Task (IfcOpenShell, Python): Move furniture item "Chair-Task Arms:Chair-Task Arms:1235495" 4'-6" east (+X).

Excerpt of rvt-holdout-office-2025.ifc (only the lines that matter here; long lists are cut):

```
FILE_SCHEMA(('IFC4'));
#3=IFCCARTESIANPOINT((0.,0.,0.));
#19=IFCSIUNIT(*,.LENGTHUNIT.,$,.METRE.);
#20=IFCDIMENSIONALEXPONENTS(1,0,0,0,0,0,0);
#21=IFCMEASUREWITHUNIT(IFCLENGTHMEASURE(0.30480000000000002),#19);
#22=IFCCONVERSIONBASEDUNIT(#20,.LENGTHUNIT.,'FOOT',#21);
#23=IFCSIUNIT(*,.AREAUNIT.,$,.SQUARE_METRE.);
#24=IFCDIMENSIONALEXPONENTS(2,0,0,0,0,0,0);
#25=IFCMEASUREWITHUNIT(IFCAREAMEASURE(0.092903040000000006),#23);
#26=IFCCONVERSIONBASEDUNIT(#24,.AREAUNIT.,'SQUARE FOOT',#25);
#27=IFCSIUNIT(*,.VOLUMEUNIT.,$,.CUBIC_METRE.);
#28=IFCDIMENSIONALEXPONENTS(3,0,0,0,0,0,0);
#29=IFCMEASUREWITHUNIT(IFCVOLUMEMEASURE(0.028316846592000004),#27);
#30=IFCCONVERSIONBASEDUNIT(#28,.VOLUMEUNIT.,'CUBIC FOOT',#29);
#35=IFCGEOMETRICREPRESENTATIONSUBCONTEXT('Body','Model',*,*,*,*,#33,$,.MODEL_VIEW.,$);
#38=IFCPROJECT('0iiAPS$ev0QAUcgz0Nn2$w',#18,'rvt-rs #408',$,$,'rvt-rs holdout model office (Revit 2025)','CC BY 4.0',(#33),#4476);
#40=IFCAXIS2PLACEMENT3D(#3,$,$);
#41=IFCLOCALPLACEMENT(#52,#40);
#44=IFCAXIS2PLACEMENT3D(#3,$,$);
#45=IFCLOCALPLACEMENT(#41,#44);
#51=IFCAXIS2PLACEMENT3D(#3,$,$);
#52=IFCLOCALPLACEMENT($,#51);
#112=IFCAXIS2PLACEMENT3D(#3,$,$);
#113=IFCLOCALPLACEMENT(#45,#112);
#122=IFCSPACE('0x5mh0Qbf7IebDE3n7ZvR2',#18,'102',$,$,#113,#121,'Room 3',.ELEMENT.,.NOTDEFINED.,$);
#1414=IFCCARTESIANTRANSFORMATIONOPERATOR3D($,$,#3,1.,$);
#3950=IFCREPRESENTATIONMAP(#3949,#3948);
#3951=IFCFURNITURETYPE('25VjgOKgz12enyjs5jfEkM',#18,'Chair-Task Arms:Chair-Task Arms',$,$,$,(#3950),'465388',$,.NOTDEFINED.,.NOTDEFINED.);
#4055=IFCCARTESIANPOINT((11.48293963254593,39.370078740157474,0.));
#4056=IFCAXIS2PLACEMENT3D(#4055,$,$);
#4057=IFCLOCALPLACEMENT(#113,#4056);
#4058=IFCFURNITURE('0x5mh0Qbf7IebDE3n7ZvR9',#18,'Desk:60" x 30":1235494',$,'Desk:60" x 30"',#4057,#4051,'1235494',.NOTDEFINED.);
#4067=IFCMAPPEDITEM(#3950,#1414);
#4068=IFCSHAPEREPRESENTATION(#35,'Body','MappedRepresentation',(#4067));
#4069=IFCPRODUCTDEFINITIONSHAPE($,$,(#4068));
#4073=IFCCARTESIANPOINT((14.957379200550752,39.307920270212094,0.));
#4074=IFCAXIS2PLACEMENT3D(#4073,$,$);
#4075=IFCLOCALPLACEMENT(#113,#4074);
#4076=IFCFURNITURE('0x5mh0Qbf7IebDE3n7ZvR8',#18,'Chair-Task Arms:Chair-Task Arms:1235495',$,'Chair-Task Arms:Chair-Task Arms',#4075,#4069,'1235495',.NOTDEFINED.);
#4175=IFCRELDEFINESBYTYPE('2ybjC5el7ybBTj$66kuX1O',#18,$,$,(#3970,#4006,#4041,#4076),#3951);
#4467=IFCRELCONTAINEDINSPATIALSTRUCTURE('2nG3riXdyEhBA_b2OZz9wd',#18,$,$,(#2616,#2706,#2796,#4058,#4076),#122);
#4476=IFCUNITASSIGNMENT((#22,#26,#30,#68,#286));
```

```python
import ifcopenshell
import ifcopenshell.api.geometry
import ifcopenshell.util.placement
import ifcopenshell.util.unit

model = ifcopenshell.open("rvt-holdout-office-2025.ifc")
unit_scale = ifcopenshell.util.unit.calculate_unit_scale(model)

item = model.by_guid("0x5mh0Qbf7IebDE3n7ZvR8")
matrix = ifcopenshell.util.placement.get_local_placement(item.ObjectPlacement)
matrix[0, 3] += 54 * 0.0254 / unit_scale
ifcopenshell.api.geometry.edit_object_placement(model, product=item, matrix=matrix, is_si=False)

print(ifcopenshell.util.placement.get_local_placement(item.ObjectPlacement).round(3) + 0.0)

model.write("rvt-holdout-office-2025_updated.ifc")
```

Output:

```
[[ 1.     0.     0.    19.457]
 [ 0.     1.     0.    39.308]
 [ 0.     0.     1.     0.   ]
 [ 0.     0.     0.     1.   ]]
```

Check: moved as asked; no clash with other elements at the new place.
